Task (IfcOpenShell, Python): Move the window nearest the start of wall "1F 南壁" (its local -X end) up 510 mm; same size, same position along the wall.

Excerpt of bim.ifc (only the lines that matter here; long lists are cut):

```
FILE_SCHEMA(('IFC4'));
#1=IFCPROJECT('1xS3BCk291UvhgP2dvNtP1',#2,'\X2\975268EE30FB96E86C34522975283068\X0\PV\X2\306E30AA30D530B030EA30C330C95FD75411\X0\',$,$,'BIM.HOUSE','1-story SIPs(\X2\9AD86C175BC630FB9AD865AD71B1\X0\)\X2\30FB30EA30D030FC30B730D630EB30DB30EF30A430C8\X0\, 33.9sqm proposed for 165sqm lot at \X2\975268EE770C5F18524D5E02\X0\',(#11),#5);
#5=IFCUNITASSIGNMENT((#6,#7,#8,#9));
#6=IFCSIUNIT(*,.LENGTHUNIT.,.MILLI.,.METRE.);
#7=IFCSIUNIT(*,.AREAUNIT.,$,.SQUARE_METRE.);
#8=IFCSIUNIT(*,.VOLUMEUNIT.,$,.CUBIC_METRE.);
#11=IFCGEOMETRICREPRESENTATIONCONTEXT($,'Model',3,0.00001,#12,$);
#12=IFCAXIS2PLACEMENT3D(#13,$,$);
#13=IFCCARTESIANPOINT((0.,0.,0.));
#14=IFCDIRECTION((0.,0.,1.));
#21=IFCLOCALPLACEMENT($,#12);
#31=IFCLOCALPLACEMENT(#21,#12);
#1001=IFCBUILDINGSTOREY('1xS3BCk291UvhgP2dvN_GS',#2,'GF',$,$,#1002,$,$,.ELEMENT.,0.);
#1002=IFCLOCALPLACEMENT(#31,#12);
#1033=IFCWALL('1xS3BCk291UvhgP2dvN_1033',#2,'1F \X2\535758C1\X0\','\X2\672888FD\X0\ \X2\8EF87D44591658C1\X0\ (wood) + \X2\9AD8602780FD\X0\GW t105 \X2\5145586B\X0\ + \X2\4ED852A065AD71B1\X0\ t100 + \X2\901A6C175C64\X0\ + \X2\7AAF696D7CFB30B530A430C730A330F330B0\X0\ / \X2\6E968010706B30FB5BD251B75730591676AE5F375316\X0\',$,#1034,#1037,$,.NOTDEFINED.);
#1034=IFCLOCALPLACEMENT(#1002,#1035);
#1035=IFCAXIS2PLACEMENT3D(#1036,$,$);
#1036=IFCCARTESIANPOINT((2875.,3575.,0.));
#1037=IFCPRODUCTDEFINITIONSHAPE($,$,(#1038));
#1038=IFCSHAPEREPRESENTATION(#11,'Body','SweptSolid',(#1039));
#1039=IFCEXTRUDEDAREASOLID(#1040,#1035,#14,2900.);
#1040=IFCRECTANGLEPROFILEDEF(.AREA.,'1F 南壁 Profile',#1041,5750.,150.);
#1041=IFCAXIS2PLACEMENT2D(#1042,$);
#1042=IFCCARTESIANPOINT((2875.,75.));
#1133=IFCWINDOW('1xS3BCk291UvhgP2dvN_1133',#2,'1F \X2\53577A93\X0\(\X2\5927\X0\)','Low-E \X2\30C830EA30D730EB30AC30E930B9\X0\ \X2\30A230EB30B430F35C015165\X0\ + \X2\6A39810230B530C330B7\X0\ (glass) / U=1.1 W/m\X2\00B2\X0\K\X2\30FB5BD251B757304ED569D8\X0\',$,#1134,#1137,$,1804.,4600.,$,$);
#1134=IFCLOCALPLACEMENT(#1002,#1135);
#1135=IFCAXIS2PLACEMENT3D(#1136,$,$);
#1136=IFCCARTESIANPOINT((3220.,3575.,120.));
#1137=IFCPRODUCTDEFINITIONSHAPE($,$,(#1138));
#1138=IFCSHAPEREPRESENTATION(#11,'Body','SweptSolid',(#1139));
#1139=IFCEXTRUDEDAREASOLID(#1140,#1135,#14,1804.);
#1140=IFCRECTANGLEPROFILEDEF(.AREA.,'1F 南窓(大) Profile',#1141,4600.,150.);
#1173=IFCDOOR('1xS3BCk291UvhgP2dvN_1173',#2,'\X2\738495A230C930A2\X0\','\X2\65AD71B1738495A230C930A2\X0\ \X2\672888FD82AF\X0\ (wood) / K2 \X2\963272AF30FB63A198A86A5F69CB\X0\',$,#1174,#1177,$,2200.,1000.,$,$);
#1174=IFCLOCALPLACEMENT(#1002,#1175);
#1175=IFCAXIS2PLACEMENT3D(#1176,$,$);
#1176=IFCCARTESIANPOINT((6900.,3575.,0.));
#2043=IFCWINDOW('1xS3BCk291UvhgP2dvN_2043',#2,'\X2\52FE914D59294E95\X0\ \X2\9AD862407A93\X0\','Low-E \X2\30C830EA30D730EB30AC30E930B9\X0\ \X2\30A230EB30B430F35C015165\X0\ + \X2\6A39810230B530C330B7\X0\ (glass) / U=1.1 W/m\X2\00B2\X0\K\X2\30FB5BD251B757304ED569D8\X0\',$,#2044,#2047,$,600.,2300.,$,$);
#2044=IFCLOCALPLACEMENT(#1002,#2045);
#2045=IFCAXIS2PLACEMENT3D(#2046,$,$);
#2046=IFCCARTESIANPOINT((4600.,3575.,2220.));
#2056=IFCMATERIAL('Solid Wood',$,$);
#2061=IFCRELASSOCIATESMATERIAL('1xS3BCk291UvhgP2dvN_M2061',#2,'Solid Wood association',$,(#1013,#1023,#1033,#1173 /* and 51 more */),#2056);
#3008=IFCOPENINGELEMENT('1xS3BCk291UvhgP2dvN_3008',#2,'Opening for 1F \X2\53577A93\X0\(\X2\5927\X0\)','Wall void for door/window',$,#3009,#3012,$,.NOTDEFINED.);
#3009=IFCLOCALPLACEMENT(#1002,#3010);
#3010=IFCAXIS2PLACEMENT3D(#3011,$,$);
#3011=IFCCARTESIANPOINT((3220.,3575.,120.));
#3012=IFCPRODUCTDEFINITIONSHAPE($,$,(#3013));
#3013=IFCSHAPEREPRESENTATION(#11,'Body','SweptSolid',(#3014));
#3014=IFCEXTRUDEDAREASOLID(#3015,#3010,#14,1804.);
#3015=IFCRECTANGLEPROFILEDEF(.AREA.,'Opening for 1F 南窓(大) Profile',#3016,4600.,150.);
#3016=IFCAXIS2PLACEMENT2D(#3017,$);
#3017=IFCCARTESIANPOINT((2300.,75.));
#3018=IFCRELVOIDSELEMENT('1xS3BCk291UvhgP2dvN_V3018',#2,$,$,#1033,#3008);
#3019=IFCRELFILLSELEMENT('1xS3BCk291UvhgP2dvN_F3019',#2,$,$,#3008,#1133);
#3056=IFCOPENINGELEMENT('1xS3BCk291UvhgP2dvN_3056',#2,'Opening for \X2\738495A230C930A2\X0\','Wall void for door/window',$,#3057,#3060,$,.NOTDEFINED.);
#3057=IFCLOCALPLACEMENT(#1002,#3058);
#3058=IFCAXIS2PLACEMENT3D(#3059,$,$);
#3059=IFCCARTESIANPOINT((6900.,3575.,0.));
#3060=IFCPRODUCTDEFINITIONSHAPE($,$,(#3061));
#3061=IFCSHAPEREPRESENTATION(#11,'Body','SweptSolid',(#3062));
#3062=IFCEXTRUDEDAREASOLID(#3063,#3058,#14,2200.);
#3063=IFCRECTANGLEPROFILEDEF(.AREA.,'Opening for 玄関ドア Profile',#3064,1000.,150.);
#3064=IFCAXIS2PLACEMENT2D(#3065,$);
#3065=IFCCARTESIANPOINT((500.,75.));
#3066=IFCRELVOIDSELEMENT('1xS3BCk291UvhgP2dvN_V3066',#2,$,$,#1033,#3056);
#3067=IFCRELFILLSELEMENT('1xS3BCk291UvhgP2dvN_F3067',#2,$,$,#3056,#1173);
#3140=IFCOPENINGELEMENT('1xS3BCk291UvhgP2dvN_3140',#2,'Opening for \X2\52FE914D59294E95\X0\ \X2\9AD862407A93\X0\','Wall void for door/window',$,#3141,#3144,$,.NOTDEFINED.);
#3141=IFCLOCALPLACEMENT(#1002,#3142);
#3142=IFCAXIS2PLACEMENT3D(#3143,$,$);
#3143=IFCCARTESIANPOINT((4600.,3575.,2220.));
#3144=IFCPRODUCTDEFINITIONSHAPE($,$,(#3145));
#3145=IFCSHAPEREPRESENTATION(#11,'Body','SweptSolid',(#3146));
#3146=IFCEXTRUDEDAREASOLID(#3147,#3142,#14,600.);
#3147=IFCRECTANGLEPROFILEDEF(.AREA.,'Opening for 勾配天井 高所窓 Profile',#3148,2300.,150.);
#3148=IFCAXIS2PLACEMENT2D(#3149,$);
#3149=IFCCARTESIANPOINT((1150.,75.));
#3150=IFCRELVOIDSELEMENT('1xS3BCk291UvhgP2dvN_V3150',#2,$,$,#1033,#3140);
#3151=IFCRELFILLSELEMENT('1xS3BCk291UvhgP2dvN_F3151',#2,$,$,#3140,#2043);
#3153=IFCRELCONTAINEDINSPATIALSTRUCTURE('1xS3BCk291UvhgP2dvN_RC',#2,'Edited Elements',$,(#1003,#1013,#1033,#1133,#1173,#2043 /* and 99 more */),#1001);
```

```python
import numpy as np
import ifcopenshell
import ifcopenshell.api.geometry
import ifcopenshell.util.placement
import ifcopenshell.util.unit

model = ifcopenshell.open("bim.ifc")
unit_scale = ifcopenshell.util.unit.calculate_unit_scale(model)

window = model.by_id(1133)
opening = window.FillsVoids[0].RelatingOpeningElement
dz = 0.51 / unit_scale

shift = np.array([0.0, 0.0, dz])
# The window is not placed relative to its opening, so move both.
for product in (opening, window):
    matrix = ifcopenshell.util.placement.get_local_placement(product.ObjectPlacement)
    matrix[:3, 3] += shift
    ifcopenshell.api.geometry.edit_object_placement(model, product=product, matrix=matrix, is_si=False)

print(f"moved by {dz * unit_scale:+.3f} m")

model.write("bim_v2.ifc")
```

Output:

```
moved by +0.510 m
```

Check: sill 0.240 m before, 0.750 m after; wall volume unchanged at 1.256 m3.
